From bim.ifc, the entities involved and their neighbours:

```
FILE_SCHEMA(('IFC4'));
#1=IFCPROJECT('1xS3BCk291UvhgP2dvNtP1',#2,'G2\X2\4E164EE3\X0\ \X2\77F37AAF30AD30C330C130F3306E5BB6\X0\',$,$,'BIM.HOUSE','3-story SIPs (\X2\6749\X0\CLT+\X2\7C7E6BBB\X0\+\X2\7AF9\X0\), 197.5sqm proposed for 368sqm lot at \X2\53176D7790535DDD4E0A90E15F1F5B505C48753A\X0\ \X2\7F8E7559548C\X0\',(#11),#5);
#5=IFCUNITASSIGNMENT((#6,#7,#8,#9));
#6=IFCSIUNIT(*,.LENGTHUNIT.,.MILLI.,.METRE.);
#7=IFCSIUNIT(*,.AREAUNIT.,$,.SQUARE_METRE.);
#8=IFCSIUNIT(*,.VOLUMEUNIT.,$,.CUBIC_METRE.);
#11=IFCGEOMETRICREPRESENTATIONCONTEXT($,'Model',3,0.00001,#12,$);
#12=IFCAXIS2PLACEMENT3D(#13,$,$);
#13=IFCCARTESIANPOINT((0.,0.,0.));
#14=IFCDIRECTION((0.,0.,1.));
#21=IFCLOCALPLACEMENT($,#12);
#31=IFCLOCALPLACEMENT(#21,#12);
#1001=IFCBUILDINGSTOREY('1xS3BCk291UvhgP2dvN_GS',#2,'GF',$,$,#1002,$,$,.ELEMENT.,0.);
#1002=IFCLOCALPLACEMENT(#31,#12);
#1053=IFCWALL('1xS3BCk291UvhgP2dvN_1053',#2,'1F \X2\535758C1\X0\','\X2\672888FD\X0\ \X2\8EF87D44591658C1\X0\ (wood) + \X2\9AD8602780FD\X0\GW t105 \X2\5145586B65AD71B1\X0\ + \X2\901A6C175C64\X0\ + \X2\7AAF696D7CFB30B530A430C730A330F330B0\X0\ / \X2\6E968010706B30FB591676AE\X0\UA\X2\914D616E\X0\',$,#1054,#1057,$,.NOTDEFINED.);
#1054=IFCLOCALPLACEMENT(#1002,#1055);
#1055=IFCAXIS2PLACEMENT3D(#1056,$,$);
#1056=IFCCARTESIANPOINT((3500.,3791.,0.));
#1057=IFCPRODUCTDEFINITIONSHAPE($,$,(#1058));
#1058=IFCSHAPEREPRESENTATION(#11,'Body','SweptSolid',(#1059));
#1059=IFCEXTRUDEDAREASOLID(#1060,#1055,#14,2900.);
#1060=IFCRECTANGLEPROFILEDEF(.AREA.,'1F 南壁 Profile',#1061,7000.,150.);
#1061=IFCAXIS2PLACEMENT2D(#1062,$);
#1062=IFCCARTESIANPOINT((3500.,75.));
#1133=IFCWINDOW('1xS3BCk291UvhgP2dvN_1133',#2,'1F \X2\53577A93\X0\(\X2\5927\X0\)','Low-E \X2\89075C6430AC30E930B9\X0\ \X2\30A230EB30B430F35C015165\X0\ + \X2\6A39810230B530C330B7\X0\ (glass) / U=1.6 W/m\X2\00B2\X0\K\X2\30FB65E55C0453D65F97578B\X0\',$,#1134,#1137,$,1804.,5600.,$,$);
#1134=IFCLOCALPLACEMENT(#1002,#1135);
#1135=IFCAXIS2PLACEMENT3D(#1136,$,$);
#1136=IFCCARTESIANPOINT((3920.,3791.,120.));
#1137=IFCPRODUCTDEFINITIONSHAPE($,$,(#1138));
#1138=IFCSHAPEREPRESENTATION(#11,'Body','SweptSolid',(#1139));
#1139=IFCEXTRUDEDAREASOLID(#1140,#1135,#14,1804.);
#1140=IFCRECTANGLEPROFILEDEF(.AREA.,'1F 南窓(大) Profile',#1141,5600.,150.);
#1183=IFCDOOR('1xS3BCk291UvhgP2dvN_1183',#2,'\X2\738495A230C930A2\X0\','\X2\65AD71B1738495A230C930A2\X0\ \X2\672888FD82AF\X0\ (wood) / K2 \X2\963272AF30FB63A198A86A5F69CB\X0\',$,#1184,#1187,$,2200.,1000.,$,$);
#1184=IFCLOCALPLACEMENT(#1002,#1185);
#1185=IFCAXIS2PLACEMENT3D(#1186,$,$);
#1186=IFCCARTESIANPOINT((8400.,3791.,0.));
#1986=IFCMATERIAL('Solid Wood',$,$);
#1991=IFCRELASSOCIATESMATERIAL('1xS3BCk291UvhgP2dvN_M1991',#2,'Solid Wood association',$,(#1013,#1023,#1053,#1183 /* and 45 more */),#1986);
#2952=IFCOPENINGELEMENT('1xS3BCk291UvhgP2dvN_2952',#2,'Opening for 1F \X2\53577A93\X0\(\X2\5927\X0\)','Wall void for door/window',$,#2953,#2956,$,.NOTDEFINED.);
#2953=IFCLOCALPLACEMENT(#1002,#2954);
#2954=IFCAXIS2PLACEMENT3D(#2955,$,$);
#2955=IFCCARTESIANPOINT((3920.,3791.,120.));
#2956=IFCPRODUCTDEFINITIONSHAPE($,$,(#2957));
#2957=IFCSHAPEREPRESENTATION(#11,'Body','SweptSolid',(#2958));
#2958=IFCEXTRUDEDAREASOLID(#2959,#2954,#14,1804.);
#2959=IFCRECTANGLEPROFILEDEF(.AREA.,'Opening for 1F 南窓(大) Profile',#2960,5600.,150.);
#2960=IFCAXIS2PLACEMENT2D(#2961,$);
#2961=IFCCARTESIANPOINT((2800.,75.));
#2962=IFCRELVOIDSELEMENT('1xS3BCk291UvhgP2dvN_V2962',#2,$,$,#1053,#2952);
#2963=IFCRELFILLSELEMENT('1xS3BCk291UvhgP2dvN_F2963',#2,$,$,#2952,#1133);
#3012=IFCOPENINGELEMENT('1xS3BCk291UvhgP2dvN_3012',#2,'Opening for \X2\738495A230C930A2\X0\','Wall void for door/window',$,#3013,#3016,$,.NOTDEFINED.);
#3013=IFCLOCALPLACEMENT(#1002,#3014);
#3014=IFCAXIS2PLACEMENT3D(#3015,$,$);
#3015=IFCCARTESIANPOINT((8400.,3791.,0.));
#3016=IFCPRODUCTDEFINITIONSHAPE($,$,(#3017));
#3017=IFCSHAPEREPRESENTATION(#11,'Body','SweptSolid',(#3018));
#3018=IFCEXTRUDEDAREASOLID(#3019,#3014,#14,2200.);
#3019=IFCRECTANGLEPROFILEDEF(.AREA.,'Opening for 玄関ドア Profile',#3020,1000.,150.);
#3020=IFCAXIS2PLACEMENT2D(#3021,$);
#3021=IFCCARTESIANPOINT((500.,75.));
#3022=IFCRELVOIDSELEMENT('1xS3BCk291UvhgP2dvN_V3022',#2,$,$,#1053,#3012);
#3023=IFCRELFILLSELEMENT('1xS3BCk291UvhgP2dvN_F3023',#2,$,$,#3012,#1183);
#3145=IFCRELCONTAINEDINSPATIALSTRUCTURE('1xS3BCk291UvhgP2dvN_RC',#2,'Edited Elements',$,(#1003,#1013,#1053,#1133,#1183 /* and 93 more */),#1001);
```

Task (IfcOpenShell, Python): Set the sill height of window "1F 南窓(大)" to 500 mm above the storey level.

```python
import numpy as np
import ifcopenshell
import ifcopenshell.api.geometry
import ifcopenshell.geom
import ifcopenshell.util.element
import ifcopenshell.util.placement
import ifcopenshell.util.shape
import ifcopenshell.util.unit

model = ifcopenshell.open("bim.ifc")
unit_scale = ifcopenshell.util.unit.calculate_unit_scale(model)

window = model.by_guid("1xS3BCk291UvhgP2dvN_1133")
opening = window.FillsVoids[0].RelatingOpeningElement
storey = ifcopenshell.util.element.get_container(window, ifc_class="IfcBuildingStorey")
level = ifcopenshell.util.placement.get_local_placement(storey.ObjectPlacement)[2, 3]

# The opening's origin need not be at the sill, so measure its lowest point.
shape = ifcopenshell.geom.create_shape(ifcopenshell.geom.settings(), opening)
bottom = ifcopenshell.util.shape.get_shape_bottom_elevation(shape, shape.geometry) / unit_scale
dz = level + 500.0 - bottom

shift = np.array([0.0, 0.0, dz])
# The window is not placed relative to its opening, so move both.
for product in (opening, window):
    matrix = ifcopenshell.util.placement.get_local_placement(product.ObjectPlacement)
    matrix[:3, 3] += shift
    ifcopenshell.api.geometry.edit_object_placement(model, product=product, matrix=matrix, is_si=False)

print(f"moved by {dz * unit_scale:+.3f} m")

model.write("bim_rev.ifc")
```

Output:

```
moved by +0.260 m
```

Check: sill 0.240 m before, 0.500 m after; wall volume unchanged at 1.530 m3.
